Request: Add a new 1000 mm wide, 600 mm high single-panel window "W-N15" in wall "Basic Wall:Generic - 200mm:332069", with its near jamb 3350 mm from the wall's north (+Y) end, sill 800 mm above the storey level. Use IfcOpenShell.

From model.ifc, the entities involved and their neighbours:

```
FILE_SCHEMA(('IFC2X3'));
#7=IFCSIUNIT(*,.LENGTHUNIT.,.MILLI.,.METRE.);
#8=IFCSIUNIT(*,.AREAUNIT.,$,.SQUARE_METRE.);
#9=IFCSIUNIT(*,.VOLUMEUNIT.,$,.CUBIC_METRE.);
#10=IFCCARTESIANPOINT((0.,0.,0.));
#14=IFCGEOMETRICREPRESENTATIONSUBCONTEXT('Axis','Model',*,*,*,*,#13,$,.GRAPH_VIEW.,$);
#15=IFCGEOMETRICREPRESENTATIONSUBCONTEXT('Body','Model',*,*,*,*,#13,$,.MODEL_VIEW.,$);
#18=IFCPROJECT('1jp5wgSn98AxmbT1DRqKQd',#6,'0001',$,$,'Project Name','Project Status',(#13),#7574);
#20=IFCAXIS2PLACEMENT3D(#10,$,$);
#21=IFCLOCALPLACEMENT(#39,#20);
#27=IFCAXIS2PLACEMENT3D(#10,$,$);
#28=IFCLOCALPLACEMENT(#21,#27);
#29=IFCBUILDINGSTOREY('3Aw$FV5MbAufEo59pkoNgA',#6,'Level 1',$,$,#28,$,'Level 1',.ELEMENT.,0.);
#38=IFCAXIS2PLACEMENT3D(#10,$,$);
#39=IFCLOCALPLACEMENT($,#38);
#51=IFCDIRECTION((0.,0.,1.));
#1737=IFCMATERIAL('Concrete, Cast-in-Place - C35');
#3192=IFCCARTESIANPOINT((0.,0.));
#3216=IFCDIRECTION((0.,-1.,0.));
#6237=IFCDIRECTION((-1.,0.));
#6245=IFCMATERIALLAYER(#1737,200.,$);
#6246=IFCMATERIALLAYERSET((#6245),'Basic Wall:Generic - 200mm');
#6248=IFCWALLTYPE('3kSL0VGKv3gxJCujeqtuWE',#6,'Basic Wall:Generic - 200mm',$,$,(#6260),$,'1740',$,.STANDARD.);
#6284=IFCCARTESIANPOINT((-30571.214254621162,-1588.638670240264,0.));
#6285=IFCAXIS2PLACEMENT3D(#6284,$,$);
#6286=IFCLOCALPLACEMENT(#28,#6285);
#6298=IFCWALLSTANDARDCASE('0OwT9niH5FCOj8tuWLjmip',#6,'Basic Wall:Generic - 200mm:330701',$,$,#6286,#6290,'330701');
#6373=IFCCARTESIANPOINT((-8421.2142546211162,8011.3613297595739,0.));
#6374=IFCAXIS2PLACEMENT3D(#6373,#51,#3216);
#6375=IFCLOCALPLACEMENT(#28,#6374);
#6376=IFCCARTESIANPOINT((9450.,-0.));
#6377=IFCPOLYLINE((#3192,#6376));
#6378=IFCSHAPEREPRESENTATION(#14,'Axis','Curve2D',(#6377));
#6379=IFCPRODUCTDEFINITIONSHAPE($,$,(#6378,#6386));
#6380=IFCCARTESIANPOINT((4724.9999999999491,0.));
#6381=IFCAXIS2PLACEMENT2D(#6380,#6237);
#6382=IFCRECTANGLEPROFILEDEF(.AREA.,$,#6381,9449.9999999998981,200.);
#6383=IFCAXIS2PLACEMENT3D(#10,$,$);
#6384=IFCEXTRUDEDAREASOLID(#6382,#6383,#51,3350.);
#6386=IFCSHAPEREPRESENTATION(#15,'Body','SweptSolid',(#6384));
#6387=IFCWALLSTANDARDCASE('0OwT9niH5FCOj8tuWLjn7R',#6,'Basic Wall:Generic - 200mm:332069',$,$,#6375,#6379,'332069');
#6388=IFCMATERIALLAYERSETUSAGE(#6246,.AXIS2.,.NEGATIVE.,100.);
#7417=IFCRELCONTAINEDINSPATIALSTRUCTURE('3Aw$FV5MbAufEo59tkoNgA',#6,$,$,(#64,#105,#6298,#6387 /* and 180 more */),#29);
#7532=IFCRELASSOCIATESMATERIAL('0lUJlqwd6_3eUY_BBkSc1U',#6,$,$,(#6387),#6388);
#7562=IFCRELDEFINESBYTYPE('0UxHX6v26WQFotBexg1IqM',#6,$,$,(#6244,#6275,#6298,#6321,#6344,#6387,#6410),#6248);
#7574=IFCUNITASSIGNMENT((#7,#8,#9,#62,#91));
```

```python
import numpy as np
import ifcopenshell
import ifcopenshell.api.feature
import ifcopenshell.api.geometry
import ifcopenshell.api.root
import ifcopenshell.api.spatial
import ifcopenshell.api.type
import ifcopenshell.geom
import ifcopenshell.util.element
import ifcopenshell.util.placement
import ifcopenshell.util.representation
import ifcopenshell.util.shape
import ifcopenshell.util.unit

model = ifcopenshell.open("model.ifc")
unit_scale = ifcopenshell.util.unit.calculate_unit_scale(model)
settings = ifcopenshell.geom.settings()


def volume(element):
    """Net volume in cubic metres, openings subtracted."""
    shape = ifcopenshell.geom.create_shape(settings, element)
    return ifcopenshell.util.shape.get_volume(shape.geometry)


wall = model.by_id(6387)
storey = ifcopenshell.util.element.get_container(wall, ifc_class="IfcBuildingStorey")
context = ifcopenshell.util.representation.get_context(model, "Model", "Body", "MODEL_VIEW")
before = volume(wall)

width, height, from_end, sill = 1, 0.6, 3.35, 0.8  # metres

# The wall runs along its own X axis, and the end named is its -X end.
wall_shape = ifcopenshell.geom.create_shape(settings, wall)
x, y, z = ifcopenshell.util.shape.get_vertices(wall_shape.geometry).T
start = x.min() + from_end
face, thickness = float(y.min()), float(y.max() - y.min())
wall_matrix = ifcopenshell.util.placement.get_local_placement(wall.ObjectPlacement)
level = ifcopenshell.util.placement.get_local_placement(storey.ObjectPlacement)[2, 3]


def in_wall(x, y):
    """Placement at x, y metres in the wall's axes, at sill height."""
    matrix = wall_matrix.copy()
    matrix[:, 3] = wall_matrix @ np.array([x / unit_scale, y / unit_scale, 0.0, 1.0])
    matrix[2, 3] = level + sill / unit_scale
    return matrix


# Opening: a box that overshoots both wall faces by 50 mm.
opening = ifcopenshell.api.root.create_entity(model, ifc_class="IfcOpeningElement")
box = ifcopenshell.api.geometry.add_wall_representation(
    model, context=context, length=width, height=height, thickness=thickness + 0.1
)
ifcopenshell.api.geometry.assign_representation(model, product=opening, representation=box)
ifcopenshell.api.geometry.edit_object_placement(model, product=opening, matrix=in_wall(start, face - 0.05), is_si=False)
ifcopenshell.api.feature.add_feature(model, feature=opening, element=wall)

window = ifcopenshell.api.root.create_entity(model, ifc_class="IfcWindow", name="W-N15")
window.OverallWidth, window.OverallHeight = width / unit_scale, height / unit_scale
body = ifcopenshell.api.geometry.add_window_representation(
    model,
    context=context,
    overall_width=window.OverallWidth,
    overall_height=window.OverallHeight,
    partition_type="SINGLE_PANEL",
)
ifcopenshell.api.geometry.assign_representation(model, product=window, representation=body)
ifcopenshell.api.spatial.assign_container(model, products=[window], relating_structure=storey)
fills = ifcopenshell.api.feature.add_filling(model, opening=opening, element=window)
fills.OwnerHistory = window.OwnerHistory  # required in IFC2X3

# IFC2X3 keeps the operation on the window style.
style = ifcopenshell.api.root.create_entity(model, ifc_class="IfcWindowStyle", name="W-N15")
style.OperationType, style.ConstructionType = "SINGLE_PANEL", "NOTDEFINED"
style.ParameterTakesPrecedence = style.Sizeable = False
ifcopenshell.api.type.assign_type(model, related_objects=[window], relating_type=style)

# Centre the window in the wall's thickness.
ifcopenshell.api.geometry.edit_object_placement(model, product=window, matrix=in_wall(start, face), is_si=False)
window_shape = ifcopenshell.geom.create_shape(settings, window)
depth = ifcopenshell.util.shape.get_vertices(window_shape.geometry)[:, 1]
offset = face + thickness / 2 - (depth.min() + depth.max()) / 2
ifcopenshell.api.geometry.edit_object_placement(model, product=window, matrix=in_wall(start, offset), is_si=False)

after = volume(wall)

print(f"wall volume {before:.3f} -> {after:.3f} m3")

model.write("model_rev.ifc")
```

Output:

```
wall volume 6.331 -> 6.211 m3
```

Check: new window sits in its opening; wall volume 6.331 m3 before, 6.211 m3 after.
